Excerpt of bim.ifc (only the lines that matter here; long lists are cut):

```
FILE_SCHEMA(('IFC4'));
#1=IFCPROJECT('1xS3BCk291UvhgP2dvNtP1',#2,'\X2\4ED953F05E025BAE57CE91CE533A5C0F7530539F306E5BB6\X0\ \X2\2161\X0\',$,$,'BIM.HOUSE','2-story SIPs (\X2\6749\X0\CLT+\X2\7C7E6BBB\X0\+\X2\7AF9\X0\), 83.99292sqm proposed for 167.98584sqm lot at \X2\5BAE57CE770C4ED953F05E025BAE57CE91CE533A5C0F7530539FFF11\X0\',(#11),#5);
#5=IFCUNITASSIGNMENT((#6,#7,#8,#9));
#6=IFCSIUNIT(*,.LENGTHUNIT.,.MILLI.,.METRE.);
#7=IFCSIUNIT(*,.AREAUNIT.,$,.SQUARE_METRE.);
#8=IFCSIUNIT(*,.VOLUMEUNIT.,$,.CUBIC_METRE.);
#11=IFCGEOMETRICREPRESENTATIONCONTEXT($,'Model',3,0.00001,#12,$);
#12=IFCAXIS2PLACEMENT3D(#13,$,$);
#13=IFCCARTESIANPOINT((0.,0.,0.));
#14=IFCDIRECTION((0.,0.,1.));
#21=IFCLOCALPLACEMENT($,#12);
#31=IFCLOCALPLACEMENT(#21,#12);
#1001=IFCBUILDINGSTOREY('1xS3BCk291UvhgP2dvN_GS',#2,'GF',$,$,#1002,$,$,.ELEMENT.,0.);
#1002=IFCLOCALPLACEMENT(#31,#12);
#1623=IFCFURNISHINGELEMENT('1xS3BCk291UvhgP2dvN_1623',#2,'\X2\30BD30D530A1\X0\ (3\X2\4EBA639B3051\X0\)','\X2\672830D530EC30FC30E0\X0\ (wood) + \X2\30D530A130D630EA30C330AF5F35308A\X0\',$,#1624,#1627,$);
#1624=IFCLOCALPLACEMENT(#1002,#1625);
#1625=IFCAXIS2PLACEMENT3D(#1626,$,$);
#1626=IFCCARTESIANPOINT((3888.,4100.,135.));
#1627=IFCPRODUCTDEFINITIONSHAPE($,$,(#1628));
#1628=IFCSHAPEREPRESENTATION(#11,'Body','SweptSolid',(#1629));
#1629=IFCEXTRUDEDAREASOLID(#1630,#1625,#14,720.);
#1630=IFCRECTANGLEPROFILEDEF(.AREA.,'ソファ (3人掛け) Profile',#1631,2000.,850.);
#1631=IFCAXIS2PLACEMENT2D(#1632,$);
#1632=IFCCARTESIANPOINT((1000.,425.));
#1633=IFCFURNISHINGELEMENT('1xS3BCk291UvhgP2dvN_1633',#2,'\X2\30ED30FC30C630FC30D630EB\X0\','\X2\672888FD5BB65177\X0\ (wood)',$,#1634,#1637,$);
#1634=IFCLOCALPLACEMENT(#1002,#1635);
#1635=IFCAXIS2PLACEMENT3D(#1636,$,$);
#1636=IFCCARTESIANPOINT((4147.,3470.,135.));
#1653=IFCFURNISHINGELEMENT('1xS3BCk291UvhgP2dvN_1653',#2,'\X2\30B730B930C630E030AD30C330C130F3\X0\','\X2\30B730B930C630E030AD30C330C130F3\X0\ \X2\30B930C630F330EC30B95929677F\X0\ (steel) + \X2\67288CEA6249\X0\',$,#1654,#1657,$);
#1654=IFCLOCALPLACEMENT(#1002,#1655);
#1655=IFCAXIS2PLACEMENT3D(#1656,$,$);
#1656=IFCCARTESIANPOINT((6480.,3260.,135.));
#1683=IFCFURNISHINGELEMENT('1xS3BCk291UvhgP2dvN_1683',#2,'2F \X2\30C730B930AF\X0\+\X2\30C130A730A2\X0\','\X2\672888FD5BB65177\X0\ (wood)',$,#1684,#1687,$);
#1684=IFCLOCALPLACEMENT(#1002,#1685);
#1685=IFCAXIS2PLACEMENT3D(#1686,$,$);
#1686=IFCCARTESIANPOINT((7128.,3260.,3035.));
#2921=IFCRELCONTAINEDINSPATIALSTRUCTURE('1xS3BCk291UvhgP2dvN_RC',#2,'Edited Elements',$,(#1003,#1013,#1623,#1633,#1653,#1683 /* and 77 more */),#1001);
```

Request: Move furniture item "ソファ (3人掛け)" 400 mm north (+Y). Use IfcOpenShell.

```python
import ifcopenshell
import ifcopenshell.api.geometry
import ifcopenshell.util.placement
import ifcopenshell.util.unit

model = ifcopenshell.open("bim.ifc")
unit_scale = ifcopenshell.util.unit.calculate_unit_scale(model)

item = model.by_id(1623)
matrix = ifcopenshell.util.placement.get_local_placement(item.ObjectPlacement)
matrix[1, 3] += 0.4 / unit_scale
ifcopenshell.api.geometry.edit_object_placement(model, product=item, matrix=matrix, is_si=False)

print(ifcopenshell.util.placement.get_local_placement(item.ObjectPlacement).round(3) + 0.0)

model.write("bim_edited.ifc")
```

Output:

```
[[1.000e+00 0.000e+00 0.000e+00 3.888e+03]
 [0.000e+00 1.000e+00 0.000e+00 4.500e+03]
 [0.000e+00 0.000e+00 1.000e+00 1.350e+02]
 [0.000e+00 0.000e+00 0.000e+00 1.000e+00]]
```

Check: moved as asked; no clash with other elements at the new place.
